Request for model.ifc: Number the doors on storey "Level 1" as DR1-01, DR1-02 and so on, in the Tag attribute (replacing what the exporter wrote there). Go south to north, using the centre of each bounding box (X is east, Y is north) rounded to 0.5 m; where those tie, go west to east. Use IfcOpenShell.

First a look at what the model holds.

```python
import ifcopenshell
import ifcopenshell.util.element
import ifcopenshell.util.placement

model = ifcopenshell.open("model.ifc")
print(model.schema)
storey = next(s for s in model.by_type("IfcBuildingStorey") if s.Name == "Level 1")
doors = [e for e in ifcopenshell.util.element.get_decomposition(storey) if e.is_a("IfcDoor")]
for e in sorted(doors, key=lambda e: e.id()):
    origin = ifcopenshell.util.placement.get_local_placement(e.ObjectPlacement)[:3, 3]
    print(e.id(), e.Tag, e.Name, origin.round(2) + 0.0, sep=" | ")
```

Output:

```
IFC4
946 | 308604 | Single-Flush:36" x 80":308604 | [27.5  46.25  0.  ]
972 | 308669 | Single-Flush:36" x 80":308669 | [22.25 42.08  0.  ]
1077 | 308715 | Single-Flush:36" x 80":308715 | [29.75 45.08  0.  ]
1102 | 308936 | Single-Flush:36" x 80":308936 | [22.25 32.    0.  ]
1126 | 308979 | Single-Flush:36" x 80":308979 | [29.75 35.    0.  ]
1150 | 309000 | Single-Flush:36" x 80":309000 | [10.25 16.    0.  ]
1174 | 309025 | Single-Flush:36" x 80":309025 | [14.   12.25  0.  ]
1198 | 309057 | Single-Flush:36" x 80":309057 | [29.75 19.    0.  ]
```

```python
import ifcopenshell
import ifcopenshell.geom
import ifcopenshell.util.element
import ifcopenshell.util.shape

model = ifcopenshell.open("model.ifc")
settings = ifcopenshell.geom.settings()
settings.set("use-world-coords", True)


def centre(element):
    shape = ifcopenshell.geom.create_shape(settings, element)
    return ifcopenshell.util.shape.get_bbox_centroid(shape.geometry)


storey = next(s for s in model.by_type("IfcBuildingStorey") if s.Name == "Level 1")
doors = [e for e in ifcopenshell.util.element.get_decomposition(storey) if e.is_a("IfcDoor")]

# Insertion points can sit at a corner or the storey origin, so sort by the geometry (in metres).
centres = {e: centre(e) for e in doors}
doors.sort(key=lambda e: (round(centres[e][1] / 0.5), centres[e][0]))

for i, e in enumerate(doors, start=1):
    number = f"DR1-{i:02d}"
    e.Tag = number
    print(e.id(), number)

model.write("model_v2.ifc")
```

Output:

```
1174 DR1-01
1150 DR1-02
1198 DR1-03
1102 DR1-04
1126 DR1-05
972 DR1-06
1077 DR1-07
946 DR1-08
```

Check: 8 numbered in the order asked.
